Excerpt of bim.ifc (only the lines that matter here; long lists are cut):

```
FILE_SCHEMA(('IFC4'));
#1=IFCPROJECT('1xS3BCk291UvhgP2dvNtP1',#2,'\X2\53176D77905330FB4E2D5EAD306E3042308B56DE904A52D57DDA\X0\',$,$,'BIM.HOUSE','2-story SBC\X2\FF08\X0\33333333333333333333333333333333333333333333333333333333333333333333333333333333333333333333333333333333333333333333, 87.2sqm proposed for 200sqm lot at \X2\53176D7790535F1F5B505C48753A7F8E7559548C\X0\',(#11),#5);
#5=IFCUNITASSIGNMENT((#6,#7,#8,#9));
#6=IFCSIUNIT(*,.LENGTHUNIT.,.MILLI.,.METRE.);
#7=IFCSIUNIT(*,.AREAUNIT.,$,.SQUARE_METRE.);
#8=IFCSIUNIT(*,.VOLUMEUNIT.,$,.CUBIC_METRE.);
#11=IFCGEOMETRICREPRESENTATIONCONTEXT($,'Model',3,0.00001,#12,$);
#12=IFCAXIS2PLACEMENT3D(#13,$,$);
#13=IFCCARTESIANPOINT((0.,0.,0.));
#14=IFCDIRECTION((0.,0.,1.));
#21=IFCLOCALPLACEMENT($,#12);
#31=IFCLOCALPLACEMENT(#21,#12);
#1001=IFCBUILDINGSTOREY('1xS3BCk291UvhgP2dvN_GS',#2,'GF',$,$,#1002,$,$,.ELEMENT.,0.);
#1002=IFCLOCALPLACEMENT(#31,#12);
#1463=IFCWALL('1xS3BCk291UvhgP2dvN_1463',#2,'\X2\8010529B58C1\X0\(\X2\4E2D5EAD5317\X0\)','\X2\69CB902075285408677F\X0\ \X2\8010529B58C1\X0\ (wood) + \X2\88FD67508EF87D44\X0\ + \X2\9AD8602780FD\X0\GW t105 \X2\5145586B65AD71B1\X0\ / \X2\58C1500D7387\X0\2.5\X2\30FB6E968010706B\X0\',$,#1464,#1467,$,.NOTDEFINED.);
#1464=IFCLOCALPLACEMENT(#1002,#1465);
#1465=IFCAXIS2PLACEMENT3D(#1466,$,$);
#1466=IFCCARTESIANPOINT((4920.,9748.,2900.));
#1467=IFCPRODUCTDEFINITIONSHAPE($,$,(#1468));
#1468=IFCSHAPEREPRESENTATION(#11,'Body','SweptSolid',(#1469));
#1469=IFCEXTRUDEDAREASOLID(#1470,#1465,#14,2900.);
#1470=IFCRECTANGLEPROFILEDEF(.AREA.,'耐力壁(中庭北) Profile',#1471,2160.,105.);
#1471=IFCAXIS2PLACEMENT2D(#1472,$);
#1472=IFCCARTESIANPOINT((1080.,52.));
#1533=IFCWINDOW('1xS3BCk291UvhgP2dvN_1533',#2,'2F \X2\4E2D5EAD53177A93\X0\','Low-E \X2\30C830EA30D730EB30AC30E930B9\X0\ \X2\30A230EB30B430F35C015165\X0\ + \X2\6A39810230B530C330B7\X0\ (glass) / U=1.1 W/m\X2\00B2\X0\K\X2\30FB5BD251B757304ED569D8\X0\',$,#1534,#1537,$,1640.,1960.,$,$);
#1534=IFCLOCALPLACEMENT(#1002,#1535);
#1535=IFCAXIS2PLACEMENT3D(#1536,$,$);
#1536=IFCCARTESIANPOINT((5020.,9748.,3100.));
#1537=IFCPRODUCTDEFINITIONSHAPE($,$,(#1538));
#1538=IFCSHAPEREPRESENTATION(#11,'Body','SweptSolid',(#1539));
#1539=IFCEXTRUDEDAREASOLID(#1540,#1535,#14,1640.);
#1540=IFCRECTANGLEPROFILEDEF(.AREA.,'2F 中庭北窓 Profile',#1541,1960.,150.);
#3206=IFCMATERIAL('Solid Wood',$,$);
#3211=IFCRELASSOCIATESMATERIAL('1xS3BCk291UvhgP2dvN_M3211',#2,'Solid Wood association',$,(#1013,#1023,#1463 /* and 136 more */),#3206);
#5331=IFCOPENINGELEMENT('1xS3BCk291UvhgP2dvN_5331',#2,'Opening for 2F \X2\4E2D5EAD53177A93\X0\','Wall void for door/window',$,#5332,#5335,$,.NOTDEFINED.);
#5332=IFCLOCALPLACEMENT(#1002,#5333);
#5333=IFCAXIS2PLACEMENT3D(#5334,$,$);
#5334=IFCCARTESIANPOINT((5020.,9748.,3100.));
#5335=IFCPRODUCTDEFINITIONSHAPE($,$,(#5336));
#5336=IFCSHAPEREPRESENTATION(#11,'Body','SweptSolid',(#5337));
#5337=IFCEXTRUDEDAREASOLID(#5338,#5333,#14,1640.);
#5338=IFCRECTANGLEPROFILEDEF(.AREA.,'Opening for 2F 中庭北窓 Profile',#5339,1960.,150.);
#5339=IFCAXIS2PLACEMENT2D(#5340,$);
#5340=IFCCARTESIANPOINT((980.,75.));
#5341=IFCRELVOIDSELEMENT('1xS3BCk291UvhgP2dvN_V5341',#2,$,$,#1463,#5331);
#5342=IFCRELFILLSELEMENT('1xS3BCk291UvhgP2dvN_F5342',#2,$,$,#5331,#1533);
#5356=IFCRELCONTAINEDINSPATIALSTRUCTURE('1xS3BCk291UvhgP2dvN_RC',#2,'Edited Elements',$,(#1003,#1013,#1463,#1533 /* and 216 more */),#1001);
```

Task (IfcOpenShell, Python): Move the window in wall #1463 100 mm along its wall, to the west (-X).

```python
import ifcopenshell
import ifcopenshell.api.geometry
import ifcopenshell.util.placement
import ifcopenshell.util.unit

model = ifcopenshell.open("bim.ifc")
unit_scale = ifcopenshell.util.unit.calculate_unit_scale(model)

window = model.by_guid("1xS3BCk291UvhgP2dvN_1533")
opening = window.FillsVoids[0].RelatingOpeningElement
wall = opening.VoidsElements[0].RelatingBuildingElement

wall_matrix = ifcopenshell.util.placement.get_local_placement(wall.ObjectPlacement)
shift = wall_matrix[:3, 0] * -0.1 / unit_scale
before = ifcopenshell.util.placement.get_local_placement(window.ObjectPlacement)[:3, 3].copy()

# The window is not placed relative to its opening, so move both.
for product in (opening, window):
    matrix = ifcopenshell.util.placement.get_local_placement(product.ObjectPlacement)
    matrix[:3, 3] += shift
    ifcopenshell.api.geometry.edit_object_placement(model, product=product, matrix=matrix, is_si=False)

after = ifcopenshell.util.placement.get_local_placement(window.ObjectPlacement)[:3, 3]
print("window moved by", (after - before).round(3) + 0.0)

model.write("bim_rev.ifc")
```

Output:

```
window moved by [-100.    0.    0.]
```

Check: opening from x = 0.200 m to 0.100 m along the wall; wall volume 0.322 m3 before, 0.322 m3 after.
